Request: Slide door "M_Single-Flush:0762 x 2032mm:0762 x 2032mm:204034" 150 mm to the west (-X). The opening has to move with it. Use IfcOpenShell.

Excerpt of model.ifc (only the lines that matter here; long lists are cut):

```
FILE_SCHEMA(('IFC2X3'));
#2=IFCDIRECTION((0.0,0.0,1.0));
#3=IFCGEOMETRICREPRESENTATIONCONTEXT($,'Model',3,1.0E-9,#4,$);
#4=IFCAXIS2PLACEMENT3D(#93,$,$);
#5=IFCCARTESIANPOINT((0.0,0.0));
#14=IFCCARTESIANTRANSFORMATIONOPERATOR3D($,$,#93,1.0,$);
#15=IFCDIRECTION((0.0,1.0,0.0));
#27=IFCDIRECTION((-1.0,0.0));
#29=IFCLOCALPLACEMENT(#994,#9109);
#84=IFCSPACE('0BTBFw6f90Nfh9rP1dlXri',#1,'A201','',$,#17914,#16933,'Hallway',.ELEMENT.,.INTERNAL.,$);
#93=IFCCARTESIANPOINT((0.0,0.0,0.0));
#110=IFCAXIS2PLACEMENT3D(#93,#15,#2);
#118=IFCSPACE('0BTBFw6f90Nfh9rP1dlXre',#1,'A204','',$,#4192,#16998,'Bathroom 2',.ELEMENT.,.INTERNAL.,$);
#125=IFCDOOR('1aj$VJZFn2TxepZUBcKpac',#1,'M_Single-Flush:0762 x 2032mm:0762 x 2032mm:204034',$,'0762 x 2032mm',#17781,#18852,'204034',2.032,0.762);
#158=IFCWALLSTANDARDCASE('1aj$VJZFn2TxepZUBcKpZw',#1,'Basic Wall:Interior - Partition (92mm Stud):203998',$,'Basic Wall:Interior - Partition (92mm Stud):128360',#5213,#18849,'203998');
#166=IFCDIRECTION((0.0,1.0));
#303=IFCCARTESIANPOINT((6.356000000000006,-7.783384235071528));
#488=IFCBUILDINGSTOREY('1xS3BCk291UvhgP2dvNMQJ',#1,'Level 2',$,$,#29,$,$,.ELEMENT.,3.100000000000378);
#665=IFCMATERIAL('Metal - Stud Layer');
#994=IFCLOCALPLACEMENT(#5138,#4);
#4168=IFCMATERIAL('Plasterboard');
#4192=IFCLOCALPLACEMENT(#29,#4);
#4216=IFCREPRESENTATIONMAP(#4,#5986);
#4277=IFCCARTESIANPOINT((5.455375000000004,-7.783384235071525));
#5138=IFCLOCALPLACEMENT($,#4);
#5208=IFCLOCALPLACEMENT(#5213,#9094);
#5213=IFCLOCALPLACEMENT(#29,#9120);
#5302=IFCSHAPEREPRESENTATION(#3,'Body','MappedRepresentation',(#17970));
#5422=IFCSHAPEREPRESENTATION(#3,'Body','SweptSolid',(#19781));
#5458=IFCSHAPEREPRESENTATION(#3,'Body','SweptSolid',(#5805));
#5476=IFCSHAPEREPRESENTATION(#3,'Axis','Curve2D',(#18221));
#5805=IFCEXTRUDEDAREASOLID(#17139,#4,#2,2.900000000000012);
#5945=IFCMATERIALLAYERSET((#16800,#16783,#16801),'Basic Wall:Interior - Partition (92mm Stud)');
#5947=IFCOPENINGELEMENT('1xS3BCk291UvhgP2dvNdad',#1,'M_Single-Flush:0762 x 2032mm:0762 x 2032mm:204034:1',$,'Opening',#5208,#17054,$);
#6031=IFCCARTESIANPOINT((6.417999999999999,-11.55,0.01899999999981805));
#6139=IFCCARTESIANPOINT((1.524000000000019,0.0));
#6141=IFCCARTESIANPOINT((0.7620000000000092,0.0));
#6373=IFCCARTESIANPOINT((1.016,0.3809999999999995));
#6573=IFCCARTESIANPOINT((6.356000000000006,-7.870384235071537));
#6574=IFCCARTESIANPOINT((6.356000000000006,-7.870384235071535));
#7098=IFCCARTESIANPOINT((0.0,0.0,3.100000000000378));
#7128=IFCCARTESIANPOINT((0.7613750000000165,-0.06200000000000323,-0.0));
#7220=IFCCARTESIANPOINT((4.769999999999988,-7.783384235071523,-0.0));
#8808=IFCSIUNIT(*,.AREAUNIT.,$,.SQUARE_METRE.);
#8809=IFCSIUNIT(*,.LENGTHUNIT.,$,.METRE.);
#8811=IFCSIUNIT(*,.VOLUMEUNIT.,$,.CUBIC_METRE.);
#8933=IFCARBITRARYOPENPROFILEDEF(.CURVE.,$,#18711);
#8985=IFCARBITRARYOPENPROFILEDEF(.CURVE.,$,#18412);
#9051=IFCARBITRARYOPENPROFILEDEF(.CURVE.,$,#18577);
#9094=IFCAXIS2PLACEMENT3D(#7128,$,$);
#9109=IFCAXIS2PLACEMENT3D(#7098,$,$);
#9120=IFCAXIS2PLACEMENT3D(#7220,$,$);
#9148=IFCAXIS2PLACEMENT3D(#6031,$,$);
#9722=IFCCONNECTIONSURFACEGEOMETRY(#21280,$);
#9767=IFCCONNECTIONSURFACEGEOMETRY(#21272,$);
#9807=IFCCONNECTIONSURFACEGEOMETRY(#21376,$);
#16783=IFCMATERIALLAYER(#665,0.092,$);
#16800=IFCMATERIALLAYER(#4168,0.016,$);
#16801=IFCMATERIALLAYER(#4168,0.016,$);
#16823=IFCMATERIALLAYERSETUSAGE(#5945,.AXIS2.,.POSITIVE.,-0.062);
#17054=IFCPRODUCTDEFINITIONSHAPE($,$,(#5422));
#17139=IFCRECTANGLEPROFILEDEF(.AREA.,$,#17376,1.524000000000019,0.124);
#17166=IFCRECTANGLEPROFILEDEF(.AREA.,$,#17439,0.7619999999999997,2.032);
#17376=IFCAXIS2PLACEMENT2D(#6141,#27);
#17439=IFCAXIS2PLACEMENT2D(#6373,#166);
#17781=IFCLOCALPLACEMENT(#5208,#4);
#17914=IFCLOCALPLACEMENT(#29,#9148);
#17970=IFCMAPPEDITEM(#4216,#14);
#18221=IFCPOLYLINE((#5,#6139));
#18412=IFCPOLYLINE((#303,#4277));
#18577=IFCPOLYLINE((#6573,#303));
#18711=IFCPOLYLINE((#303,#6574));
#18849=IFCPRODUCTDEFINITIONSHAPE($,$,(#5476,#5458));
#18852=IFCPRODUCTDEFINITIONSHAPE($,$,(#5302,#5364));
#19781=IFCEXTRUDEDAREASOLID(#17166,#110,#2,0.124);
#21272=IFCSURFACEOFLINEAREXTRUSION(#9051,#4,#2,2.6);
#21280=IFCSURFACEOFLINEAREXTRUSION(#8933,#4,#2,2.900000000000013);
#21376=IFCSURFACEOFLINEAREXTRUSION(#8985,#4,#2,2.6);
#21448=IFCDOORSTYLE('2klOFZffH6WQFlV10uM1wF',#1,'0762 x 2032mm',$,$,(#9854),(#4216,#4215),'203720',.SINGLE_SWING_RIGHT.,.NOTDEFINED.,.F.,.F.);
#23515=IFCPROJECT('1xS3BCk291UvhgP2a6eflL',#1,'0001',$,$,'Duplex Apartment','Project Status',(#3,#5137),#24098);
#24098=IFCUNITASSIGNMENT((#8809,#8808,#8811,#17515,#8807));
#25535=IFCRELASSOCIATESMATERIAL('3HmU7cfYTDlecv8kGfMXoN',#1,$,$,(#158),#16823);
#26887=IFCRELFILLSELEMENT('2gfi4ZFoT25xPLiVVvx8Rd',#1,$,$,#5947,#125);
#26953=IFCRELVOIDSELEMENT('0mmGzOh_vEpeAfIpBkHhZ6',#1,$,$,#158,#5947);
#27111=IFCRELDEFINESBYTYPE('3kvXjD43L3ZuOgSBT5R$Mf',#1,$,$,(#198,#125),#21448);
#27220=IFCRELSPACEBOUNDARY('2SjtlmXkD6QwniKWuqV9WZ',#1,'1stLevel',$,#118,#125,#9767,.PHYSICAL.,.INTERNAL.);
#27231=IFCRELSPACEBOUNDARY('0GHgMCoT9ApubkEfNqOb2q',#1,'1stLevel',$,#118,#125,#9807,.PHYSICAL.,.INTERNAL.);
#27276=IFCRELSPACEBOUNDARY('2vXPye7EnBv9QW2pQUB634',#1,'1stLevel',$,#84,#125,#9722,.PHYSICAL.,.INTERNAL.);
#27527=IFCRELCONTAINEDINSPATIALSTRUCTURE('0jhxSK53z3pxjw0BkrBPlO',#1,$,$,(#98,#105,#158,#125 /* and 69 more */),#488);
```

```python
import numpy as np
import ifcopenshell
import ifcopenshell.api.geometry
import ifcopenshell.util.placement
import ifcopenshell.util.unit

model = ifcopenshell.open("model.ifc")
unit_scale = ifcopenshell.util.unit.calculate_unit_scale(model)

door = model.by_id(125)
opening = door.FillsVoids[0].RelatingOpeningElement
wall = opening.VoidsElements[0].RelatingBuildingElement

wall_matrix = ifcopenshell.util.placement.get_local_placement(wall.ObjectPlacement)
shift = wall_matrix[:3, 0] * -0.15 / unit_scale
before = ifcopenshell.util.placement.get_local_placement(door.ObjectPlacement)[:3, 3].copy()

# The door is placed relative to its opening, so it follows when the opening moves.
matrix = ifcopenshell.util.placement.get_local_placement(opening.ObjectPlacement)
matrix[:3, 3] += shift
ifcopenshell.api.geometry.edit_object_placement(
    model, product=opening, matrix=matrix, is_si=False, should_transform_children=True
)

# Space boundary surfaces are stored in each space's coordinates; move them too.
for rel in door.ProvidesBoundaries:
    if not rel.ConnectionGeometry:
        continue
    surface = rel.ConnectionGeometry.SurfaceOnRelatingElement
    space_matrix = ifcopenshell.util.placement.get_local_placement(rel.RelatingSpace.ObjectPlacement)
    point = np.array(surface.Position.Location.Coordinates) + space_matrix[:3, :3].T @ shift
    surface.Position = model.createIfcAxis2Placement3D(
        model.createIfcCartesianPoint(point.tolist()), surface.Position.Axis, surface.Position.RefDirection
    )

after = ifcopenshell.util.placement.get_local_placement(door.ObjectPlacement)[:3, 3]
print("door moved by", (after - before).round(3) + 0.0)

model.write("model_edited.ifc")
```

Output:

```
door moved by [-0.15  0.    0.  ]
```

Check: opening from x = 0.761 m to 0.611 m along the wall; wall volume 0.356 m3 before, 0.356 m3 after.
